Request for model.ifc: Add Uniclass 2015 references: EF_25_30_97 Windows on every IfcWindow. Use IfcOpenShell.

First a look at what the model holds.

```python
import ifcopenshell

model = ifcopenshell.open("model.ifc")
print(model.schema)
print("classifications:", [c.Name for c in model.by_type("IfcClassification")])
for ifc_class in ("IfcDoor", "IfcRoof", "IfcStair", "IfcWall", "IfcWindow"):
    print(ifc_class, len(model.by_type(ifc_class)))
```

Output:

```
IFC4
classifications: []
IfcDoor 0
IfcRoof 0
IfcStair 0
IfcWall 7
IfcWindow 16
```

```python
import ifcopenshell
import ifcopenshell.api.classification

model = ifcopenshell.open("model.ifc")

system = ifcopenshell.api.classification.add_classification(model, classification="Uniclass 2015")

codes = {
    "IfcWindow": ("EF_25_30_97", "Windows"),
}
for ifc_class, (code, name) in codes.items():
    products = model.by_type(ifc_class)
    ifcopenshell.api.classification.add_reference(
        model, products=products, classification=system, identification=code, name=name
    )
    print(code, len(products))

model.write("model_edited.ifc")
```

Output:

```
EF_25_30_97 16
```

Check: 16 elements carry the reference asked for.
